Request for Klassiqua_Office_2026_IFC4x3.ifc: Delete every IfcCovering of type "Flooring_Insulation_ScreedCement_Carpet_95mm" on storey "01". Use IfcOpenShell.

First a look at what the model holds.

```python
import ifcopenshell
import ifcopenshell.util.element

model = ifcopenshell.open("Klassiqua_Office_2026_IFC4x3.ifc")
print(model.schema)
storey = next(s for s in model.by_type("IfcBuildingStorey") if s.Name == "01")
coverings = [e for e in ifcopenshell.util.element.get_decomposition(storey) if e.is_a("IfcCovering")]
seen = {}
for e in coverings:
    element_type = ifcopenshell.util.element.get_type(e)
    name = element_type.Name if element_type not in (None, e) else None
    seen[name] = seen.get(name, 0) + 1
for name, count in sorted(seen.items(), key=str):
    print(count, "x", name)
```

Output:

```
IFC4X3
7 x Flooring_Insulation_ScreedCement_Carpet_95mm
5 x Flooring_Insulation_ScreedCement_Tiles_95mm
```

```python
import ifcopenshell
import ifcopenshell.api.root
import ifcopenshell.util.element

model = ifcopenshell.open("Klassiqua_Office_2026_IFC4x3.ifc")

storey = next(s for s in model.by_type("IfcBuildingStorey") if s.Name == "01")
coverings = [e for e in ifcopenshell.util.element.get_decomposition(storey) if e.is_a("IfcCovering")]
targets = [e for e in coverings if (t := ifcopenshell.util.element.get_type(e)) not in (None, e) and t.Name == "Flooring_Insulation_ScreedCement_Carpet_95mm"]

for e in targets:
    ifcopenshell.api.root.remove_product(model, product=e)
print(len(targets), "removed")

model.write("Klassiqua_Office_2026_IFC4x3_updated.ifc")
```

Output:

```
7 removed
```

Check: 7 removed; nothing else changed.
